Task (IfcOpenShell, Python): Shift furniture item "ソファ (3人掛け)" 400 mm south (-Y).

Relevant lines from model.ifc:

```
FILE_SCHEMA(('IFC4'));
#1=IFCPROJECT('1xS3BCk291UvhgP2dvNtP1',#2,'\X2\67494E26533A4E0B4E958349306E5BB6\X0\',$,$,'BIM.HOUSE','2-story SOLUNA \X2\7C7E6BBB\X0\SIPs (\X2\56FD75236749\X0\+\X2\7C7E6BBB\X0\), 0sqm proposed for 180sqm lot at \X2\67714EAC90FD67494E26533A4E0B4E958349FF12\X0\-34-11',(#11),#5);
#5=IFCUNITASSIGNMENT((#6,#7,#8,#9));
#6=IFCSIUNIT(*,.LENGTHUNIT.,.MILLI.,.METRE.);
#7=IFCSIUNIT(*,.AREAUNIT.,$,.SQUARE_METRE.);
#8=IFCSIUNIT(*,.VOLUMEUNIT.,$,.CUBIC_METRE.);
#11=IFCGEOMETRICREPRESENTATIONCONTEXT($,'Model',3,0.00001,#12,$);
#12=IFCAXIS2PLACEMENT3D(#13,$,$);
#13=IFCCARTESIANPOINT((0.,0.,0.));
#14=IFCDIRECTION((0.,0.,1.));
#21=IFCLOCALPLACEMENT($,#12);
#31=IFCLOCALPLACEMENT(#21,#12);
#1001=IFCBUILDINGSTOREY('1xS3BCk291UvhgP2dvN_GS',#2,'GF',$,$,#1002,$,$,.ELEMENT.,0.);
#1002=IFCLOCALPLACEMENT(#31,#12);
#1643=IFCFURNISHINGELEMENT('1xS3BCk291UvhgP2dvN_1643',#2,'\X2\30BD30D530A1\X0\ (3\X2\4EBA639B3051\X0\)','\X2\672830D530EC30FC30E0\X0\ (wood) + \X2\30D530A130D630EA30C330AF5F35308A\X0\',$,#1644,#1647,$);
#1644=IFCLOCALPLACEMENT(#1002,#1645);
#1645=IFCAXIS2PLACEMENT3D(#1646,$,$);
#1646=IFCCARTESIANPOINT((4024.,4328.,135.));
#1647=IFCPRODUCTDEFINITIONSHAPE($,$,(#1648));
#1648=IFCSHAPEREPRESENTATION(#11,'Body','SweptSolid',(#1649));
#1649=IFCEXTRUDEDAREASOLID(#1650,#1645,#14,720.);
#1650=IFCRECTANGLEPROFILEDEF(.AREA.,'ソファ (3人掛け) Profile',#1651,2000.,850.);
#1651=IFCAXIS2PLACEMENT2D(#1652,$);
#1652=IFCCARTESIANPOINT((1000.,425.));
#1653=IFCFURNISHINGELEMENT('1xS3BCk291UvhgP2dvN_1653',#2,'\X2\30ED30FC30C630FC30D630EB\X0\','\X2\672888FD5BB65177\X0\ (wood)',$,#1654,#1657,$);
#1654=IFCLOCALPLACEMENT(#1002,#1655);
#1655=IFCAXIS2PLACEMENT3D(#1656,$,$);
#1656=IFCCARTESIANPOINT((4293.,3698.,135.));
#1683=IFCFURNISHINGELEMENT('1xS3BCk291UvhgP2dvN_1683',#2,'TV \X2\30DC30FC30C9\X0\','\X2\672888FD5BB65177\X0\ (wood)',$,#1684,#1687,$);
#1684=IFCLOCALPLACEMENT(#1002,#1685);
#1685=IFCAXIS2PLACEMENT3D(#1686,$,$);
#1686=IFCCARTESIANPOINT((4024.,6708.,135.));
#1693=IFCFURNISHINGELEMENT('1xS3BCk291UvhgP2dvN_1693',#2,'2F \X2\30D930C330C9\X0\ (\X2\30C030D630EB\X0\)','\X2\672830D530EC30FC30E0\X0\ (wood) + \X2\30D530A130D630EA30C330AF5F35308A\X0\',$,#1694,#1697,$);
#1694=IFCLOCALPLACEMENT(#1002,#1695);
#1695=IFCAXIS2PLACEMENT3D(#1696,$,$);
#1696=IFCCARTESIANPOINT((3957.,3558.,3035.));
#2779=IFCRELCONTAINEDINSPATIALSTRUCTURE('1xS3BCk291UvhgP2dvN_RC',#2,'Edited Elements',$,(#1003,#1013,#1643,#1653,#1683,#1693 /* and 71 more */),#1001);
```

```python
import ifcopenshell
import ifcopenshell.api.geometry
import ifcopenshell.util.placement

model = ifcopenshell.open("model.ifc")

item = model.by_id(1643)
matrix = ifcopenshell.util.placement.get_local_placement(item.ObjectPlacement)
matrix[1, 3] -= 400.0
ifcopenshell.api.geometry.edit_object_placement(model, product=item, matrix=matrix, is_si=False)

print(ifcopenshell.util.placement.get_local_placement(item.ObjectPlacement).round(3) + 0.0)

model.write("model_updated.ifc")
```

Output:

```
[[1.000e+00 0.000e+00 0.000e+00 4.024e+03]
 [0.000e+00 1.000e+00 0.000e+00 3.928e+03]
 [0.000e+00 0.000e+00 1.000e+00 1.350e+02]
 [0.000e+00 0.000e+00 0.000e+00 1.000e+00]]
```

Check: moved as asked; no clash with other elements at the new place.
